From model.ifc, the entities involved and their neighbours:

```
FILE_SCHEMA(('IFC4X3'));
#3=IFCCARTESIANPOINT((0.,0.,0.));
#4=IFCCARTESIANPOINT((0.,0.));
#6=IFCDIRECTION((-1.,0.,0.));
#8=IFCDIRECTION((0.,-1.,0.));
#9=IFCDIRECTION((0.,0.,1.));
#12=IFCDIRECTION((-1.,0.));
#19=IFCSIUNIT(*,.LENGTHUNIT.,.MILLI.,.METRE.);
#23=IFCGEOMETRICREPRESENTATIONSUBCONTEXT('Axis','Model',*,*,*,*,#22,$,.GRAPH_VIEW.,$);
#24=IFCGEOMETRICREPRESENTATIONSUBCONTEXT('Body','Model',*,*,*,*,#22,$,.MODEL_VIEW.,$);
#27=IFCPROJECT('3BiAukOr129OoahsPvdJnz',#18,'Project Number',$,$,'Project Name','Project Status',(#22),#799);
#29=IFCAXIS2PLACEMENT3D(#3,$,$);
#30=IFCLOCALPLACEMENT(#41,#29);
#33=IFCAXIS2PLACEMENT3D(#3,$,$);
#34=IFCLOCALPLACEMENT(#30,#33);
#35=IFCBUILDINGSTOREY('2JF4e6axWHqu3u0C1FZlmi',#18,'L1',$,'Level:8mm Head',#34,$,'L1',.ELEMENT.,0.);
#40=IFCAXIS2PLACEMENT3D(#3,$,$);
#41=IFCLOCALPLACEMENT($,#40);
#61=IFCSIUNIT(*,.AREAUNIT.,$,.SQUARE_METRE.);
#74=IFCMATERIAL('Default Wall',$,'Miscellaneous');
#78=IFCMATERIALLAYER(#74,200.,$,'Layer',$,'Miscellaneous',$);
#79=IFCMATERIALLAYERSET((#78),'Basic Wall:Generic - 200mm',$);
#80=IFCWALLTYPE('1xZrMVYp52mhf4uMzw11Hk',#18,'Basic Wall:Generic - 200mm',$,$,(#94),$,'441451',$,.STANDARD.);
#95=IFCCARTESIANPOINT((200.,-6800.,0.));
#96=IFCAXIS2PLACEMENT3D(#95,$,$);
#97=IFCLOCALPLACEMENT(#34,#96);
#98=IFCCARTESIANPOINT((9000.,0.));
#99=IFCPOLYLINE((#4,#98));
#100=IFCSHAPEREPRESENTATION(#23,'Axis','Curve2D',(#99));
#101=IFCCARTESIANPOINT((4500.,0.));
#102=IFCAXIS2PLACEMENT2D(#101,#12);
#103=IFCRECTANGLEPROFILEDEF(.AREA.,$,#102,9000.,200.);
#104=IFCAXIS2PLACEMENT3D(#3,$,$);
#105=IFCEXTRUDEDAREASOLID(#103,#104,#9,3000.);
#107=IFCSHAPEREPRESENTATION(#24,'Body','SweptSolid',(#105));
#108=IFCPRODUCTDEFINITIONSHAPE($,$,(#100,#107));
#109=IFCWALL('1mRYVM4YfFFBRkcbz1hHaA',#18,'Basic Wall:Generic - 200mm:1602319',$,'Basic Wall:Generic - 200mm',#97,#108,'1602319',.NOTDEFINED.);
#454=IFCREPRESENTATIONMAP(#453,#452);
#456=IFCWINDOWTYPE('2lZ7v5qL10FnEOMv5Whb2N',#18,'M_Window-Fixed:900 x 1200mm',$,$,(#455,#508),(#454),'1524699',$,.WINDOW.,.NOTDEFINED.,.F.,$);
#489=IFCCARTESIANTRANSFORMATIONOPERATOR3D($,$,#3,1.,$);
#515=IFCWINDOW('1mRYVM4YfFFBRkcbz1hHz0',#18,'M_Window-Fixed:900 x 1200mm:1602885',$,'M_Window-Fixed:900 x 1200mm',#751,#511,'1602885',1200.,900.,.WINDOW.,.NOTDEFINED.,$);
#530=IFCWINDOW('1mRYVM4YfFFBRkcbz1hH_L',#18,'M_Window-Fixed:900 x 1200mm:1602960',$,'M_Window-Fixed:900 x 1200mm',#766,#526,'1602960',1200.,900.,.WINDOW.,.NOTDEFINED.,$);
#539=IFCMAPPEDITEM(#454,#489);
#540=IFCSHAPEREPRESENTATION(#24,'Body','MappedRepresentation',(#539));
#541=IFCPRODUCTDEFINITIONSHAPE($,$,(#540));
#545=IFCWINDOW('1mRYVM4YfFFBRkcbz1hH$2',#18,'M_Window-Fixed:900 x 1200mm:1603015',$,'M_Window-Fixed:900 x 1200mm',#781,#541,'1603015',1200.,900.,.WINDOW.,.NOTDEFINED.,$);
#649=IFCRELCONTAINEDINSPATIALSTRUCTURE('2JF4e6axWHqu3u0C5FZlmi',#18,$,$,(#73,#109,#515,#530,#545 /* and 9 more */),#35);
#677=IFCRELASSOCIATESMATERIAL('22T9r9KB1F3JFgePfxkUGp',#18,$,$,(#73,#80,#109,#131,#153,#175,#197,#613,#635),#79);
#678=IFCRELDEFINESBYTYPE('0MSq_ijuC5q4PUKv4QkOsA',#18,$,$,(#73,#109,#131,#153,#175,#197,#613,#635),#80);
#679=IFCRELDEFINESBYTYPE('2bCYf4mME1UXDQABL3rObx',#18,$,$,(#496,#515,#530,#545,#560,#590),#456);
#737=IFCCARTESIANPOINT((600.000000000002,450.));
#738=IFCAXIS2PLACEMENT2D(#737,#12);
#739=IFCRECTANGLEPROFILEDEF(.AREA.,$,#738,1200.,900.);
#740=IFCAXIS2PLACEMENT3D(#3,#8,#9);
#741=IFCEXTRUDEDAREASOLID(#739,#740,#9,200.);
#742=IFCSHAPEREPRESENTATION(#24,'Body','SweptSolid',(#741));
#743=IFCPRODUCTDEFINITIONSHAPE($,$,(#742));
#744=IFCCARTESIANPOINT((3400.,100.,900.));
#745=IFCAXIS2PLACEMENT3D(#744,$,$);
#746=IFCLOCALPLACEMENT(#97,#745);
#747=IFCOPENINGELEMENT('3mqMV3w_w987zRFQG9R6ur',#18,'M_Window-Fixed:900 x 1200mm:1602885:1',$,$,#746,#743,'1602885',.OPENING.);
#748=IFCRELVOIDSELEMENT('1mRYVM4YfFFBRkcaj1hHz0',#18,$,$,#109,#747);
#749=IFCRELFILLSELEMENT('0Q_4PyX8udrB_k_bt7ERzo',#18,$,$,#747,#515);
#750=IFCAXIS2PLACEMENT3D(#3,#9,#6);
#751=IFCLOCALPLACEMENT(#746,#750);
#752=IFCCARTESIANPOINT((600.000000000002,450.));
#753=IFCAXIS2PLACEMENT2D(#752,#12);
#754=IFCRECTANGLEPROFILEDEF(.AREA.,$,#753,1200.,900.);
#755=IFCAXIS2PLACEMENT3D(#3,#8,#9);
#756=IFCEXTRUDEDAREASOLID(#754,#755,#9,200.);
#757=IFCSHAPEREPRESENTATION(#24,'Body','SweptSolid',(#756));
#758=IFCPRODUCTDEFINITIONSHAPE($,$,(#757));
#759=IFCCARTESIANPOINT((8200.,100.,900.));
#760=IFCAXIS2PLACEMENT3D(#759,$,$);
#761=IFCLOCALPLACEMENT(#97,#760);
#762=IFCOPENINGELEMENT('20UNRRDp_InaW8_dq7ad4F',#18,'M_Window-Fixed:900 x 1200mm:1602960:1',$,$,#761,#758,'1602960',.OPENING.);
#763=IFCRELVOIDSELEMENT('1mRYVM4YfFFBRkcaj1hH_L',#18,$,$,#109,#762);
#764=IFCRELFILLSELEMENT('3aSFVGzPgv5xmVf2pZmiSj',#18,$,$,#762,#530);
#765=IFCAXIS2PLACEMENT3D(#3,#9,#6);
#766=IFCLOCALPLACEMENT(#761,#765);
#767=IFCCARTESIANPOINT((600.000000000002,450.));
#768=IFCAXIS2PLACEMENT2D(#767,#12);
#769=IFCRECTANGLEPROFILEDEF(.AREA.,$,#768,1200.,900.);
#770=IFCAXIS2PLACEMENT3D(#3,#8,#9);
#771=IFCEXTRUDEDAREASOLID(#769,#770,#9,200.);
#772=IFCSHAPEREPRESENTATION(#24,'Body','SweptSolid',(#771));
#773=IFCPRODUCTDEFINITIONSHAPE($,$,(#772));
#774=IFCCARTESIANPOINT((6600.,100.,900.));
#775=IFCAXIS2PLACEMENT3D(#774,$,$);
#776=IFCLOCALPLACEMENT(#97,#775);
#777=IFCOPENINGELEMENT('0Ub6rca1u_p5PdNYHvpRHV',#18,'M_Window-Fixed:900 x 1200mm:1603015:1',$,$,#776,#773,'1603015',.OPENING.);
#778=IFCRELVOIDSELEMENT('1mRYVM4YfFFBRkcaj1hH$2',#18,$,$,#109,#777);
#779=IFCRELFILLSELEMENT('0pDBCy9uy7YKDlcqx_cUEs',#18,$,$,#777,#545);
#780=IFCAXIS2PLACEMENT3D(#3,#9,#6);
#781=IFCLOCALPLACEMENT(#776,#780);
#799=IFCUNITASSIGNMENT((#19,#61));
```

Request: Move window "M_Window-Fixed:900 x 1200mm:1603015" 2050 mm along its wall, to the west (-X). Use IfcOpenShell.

```python
import ifcopenshell
import ifcopenshell.api.geometry
import ifcopenshell.util.placement
import ifcopenshell.util.unit

model = ifcopenshell.open("model.ifc")
unit_scale = ifcopenshell.util.unit.calculate_unit_scale(model)

window = model.by_guid("1mRYVM4YfFFBRkcbz1hH$2")
opening = window.FillsVoids[0].RelatingOpeningElement
wall = opening.VoidsElements[0].RelatingBuildingElement

wall_matrix = ifcopenshell.util.placement.get_local_placement(wall.ObjectPlacement)
shift = wall_matrix[:3, 0] * -2.05 / unit_scale
before = ifcopenshell.util.placement.get_local_placement(window.ObjectPlacement)[:3, 3].copy()

# The window is placed relative to its opening, so it follows when the opening moves.
matrix = ifcopenshell.util.placement.get_local_placement(opening.ObjectPlacement)
matrix[:3, 3] += shift
ifcopenshell.api.geometry.edit_object_placement(
    model, product=opening, matrix=matrix, is_si=False, should_transform_children=True
)

after = ifcopenshell.util.placement.get_local_placement(window.ObjectPlacement)[:3, 3]
print("window moved by", (after - before).round(3) + 0.0)

model.write("model_rev.ifc")
```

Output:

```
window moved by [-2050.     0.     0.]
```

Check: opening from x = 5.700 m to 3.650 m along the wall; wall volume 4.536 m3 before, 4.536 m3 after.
